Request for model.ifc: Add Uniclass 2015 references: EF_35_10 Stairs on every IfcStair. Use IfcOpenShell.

First a look at what the model holds.

```python
import ifcopenshell

model = ifcopenshell.open("model.ifc")
print(model.schema)
print("classifications:", [c.Name for c in model.by_type("IfcClassification")])
for ifc_class in ("IfcDoor", "IfcRoof", "IfcStair", "IfcWall", "IfcWindow"):
    print(ifc_class, len(model.by_type(ifc_class)))
```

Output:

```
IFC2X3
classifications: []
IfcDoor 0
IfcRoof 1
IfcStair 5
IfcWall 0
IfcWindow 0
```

```python
import ifcopenshell
import ifcopenshell.api.classification

model = ifcopenshell.open("model.ifc")

# IFC2X3 requires Source and Edition and has no link from the project to the system.
system = model.create_entity("IfcClassification", Source="NBS", Edition="2015", Name="Uniclass 2015")

codes = {
    "IfcStair": ("EF_35_10", "Stairs"),
}
for ifc_class, (code, name) in codes.items():
    products = model.by_type(ifc_class)
    ifcopenshell.api.classification.add_reference(
        model, products=products, classification=system, identification=code, name=name
    )
    print(code, len(products))

model.write("model_v2.ifc")
```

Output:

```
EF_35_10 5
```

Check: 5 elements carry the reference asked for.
